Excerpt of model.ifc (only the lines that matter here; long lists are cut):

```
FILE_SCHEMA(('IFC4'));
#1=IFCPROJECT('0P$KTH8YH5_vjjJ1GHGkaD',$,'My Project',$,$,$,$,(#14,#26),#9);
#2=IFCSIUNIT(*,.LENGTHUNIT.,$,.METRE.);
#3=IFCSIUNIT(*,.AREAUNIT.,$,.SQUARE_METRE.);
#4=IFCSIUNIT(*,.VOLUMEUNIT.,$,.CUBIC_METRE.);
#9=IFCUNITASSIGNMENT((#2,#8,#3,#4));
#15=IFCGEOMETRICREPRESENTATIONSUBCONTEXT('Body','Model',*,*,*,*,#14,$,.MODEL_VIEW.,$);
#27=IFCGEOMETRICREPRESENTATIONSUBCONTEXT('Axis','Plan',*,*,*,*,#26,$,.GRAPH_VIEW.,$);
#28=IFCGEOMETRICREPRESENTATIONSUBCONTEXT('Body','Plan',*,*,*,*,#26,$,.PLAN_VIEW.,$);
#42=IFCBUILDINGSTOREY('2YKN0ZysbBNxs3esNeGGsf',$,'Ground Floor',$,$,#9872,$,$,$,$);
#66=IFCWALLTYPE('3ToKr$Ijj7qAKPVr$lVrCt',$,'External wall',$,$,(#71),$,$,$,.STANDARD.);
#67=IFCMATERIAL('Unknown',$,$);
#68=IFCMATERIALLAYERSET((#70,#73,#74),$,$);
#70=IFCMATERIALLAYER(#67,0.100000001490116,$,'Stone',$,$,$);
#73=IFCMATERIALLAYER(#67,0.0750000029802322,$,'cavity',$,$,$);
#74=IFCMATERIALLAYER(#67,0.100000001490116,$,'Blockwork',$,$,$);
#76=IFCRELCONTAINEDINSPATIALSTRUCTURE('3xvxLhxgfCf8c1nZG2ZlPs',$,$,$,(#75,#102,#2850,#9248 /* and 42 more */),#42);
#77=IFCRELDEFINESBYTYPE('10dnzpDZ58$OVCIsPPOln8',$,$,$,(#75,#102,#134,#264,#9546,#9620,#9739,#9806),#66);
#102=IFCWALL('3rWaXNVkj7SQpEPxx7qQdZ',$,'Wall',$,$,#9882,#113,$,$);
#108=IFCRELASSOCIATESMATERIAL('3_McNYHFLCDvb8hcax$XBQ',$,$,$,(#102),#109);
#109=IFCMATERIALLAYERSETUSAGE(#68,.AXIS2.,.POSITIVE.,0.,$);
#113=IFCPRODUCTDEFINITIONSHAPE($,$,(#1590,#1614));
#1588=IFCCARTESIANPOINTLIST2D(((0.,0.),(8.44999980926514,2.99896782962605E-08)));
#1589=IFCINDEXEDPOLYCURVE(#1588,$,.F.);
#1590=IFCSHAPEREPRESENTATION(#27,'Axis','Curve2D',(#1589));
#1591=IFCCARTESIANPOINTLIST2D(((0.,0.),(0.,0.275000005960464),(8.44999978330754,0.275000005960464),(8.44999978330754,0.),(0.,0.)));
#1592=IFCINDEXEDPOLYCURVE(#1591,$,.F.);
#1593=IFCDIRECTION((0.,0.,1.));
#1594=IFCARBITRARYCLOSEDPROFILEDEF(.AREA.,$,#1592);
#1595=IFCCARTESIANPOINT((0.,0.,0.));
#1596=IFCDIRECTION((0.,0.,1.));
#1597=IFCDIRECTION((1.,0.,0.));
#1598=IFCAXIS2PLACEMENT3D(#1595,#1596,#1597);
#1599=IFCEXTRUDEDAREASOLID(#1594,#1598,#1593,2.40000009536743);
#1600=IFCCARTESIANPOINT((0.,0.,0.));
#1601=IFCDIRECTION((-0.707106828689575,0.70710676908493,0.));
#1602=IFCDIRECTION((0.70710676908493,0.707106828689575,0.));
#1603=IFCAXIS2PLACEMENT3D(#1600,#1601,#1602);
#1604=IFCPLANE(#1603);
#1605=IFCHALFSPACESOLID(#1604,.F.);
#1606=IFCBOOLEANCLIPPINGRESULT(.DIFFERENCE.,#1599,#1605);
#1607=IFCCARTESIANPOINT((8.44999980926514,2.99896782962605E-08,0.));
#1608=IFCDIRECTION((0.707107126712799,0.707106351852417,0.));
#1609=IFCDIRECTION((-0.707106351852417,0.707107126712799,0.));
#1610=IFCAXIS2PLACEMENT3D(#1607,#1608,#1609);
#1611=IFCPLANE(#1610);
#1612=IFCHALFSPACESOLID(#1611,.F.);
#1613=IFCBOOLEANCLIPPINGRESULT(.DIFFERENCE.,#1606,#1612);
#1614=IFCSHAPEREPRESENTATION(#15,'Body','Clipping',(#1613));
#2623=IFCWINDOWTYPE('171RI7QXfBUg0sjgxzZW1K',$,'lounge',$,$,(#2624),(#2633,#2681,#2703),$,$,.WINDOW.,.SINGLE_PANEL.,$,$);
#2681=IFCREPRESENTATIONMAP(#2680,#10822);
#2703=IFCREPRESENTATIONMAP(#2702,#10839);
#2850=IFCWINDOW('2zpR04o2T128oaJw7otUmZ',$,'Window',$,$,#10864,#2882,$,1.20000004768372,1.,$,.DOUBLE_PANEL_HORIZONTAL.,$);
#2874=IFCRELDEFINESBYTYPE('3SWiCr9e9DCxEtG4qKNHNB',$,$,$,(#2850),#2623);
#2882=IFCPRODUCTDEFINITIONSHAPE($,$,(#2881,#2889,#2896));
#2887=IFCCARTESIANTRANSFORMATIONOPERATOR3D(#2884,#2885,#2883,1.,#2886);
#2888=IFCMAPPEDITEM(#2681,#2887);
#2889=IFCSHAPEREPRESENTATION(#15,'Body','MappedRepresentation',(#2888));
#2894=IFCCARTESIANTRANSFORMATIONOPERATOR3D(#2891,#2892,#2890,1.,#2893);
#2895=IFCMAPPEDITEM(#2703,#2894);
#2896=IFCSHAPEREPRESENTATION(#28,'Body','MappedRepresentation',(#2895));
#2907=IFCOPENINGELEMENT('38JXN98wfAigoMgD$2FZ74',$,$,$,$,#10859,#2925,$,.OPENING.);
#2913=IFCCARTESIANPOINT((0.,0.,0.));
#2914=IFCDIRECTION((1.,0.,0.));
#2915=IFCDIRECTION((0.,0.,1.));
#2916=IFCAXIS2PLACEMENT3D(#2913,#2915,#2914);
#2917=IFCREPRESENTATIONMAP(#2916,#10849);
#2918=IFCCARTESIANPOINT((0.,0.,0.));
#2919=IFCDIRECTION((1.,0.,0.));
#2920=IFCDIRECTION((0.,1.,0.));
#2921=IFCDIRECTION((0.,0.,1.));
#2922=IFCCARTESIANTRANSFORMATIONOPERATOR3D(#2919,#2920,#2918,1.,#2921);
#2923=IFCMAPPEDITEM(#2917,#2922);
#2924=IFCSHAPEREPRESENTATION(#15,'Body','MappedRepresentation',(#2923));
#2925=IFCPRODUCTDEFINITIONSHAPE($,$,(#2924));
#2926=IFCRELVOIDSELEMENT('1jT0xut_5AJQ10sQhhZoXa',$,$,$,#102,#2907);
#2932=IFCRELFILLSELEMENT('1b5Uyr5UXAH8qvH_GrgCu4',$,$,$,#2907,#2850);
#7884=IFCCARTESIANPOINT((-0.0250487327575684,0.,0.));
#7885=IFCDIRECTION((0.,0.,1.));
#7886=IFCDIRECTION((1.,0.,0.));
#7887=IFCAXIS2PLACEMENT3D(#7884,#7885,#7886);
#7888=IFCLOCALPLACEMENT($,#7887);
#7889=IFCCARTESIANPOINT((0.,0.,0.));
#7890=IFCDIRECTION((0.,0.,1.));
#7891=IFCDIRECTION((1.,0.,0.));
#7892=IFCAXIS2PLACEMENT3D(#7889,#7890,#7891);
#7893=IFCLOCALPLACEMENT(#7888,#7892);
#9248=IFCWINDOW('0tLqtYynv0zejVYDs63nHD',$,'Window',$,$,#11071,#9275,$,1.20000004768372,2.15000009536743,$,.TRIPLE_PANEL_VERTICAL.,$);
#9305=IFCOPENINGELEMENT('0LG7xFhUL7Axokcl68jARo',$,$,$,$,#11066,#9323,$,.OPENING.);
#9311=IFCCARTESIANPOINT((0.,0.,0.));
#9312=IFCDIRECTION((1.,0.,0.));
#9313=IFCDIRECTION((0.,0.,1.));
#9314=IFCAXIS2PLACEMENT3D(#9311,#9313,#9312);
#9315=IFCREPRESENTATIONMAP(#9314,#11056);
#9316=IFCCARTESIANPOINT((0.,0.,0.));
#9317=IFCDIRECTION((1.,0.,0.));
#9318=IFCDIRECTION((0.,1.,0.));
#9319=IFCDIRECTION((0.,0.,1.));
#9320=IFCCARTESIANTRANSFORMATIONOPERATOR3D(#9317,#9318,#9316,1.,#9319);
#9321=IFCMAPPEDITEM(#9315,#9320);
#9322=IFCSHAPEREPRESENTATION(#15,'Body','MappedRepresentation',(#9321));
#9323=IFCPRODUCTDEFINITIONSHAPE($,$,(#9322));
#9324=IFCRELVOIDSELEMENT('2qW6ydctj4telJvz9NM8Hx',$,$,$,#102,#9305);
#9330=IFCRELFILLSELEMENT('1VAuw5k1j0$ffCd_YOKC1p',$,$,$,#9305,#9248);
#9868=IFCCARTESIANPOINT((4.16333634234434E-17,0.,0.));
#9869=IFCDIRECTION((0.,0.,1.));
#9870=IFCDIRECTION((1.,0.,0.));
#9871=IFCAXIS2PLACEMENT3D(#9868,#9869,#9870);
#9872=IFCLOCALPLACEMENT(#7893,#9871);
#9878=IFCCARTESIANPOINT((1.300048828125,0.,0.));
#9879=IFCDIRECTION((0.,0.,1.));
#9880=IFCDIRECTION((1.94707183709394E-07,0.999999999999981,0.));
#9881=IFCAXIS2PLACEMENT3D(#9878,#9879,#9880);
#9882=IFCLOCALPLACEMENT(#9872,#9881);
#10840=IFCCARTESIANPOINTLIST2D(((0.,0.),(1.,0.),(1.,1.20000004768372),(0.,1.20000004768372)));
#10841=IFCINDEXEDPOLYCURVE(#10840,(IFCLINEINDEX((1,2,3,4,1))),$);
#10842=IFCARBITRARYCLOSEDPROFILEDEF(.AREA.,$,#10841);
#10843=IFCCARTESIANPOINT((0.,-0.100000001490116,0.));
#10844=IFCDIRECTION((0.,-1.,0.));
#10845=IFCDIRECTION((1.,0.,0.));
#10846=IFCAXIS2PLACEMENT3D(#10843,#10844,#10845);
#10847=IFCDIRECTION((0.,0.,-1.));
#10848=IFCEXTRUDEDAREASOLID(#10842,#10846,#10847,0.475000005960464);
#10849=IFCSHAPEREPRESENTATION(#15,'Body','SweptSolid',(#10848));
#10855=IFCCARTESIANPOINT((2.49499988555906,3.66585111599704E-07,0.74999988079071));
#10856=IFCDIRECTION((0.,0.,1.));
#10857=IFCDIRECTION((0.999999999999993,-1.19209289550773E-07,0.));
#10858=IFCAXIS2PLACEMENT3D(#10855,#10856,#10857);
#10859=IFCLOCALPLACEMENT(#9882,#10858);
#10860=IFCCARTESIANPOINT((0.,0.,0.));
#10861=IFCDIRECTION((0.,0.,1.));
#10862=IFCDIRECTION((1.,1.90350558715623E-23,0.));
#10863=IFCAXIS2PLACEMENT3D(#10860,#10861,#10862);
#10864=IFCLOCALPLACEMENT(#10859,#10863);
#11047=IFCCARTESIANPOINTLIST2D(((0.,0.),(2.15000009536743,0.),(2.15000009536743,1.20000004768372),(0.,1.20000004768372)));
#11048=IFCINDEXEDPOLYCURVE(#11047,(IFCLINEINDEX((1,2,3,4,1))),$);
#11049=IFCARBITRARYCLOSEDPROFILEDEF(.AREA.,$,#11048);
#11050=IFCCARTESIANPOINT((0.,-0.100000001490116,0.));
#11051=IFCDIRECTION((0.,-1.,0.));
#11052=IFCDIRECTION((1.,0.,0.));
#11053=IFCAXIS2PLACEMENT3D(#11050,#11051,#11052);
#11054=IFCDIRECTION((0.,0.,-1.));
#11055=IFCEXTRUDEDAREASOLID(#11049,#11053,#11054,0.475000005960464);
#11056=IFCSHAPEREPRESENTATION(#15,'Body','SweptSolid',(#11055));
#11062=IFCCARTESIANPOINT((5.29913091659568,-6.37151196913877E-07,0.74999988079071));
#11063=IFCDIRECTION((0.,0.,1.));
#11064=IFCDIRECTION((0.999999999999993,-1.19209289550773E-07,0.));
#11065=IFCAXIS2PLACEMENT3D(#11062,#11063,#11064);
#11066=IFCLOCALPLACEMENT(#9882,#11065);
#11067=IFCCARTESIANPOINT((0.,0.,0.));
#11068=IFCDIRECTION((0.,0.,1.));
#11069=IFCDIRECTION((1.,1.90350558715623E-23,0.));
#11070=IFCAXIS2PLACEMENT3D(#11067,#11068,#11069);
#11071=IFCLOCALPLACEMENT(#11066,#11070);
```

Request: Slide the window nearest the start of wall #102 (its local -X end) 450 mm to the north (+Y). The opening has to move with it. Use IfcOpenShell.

```python
import ifcopenshell
import ifcopenshell.api.geometry
import ifcopenshell.util.placement

model = ifcopenshell.open("model.ifc")

window = model.by_guid("2zpR04o2T128oaJw7otUmZ")
opening = window.FillsVoids[0].RelatingOpeningElement
wall = opening.VoidsElements[0].RelatingBuildingElement

wall_matrix = ifcopenshell.util.placement.get_local_placement(wall.ObjectPlacement)
shift = wall_matrix[:3, 0] * 0.45
before = ifcopenshell.util.placement.get_local_placement(window.ObjectPlacement)[:3, 3].copy()

# The window is placed relative to its opening, so it follows when the opening moves.
matrix = ifcopenshell.util.placement.get_local_placement(opening.ObjectPlacement)
matrix[:3, 3] += shift
ifcopenshell.api.geometry.edit_object_placement(
    model, product=opening, matrix=matrix, is_si=False, should_transform_children=True
)

after = ifcopenshell.util.placement.get_local_placement(window.ObjectPlacement)[:3, 3]
print("window moved by", (after - before).round(3) + 0.0)

model.write("model_edited.ifc")
```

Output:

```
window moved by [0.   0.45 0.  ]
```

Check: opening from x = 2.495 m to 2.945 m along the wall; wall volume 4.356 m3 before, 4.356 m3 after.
